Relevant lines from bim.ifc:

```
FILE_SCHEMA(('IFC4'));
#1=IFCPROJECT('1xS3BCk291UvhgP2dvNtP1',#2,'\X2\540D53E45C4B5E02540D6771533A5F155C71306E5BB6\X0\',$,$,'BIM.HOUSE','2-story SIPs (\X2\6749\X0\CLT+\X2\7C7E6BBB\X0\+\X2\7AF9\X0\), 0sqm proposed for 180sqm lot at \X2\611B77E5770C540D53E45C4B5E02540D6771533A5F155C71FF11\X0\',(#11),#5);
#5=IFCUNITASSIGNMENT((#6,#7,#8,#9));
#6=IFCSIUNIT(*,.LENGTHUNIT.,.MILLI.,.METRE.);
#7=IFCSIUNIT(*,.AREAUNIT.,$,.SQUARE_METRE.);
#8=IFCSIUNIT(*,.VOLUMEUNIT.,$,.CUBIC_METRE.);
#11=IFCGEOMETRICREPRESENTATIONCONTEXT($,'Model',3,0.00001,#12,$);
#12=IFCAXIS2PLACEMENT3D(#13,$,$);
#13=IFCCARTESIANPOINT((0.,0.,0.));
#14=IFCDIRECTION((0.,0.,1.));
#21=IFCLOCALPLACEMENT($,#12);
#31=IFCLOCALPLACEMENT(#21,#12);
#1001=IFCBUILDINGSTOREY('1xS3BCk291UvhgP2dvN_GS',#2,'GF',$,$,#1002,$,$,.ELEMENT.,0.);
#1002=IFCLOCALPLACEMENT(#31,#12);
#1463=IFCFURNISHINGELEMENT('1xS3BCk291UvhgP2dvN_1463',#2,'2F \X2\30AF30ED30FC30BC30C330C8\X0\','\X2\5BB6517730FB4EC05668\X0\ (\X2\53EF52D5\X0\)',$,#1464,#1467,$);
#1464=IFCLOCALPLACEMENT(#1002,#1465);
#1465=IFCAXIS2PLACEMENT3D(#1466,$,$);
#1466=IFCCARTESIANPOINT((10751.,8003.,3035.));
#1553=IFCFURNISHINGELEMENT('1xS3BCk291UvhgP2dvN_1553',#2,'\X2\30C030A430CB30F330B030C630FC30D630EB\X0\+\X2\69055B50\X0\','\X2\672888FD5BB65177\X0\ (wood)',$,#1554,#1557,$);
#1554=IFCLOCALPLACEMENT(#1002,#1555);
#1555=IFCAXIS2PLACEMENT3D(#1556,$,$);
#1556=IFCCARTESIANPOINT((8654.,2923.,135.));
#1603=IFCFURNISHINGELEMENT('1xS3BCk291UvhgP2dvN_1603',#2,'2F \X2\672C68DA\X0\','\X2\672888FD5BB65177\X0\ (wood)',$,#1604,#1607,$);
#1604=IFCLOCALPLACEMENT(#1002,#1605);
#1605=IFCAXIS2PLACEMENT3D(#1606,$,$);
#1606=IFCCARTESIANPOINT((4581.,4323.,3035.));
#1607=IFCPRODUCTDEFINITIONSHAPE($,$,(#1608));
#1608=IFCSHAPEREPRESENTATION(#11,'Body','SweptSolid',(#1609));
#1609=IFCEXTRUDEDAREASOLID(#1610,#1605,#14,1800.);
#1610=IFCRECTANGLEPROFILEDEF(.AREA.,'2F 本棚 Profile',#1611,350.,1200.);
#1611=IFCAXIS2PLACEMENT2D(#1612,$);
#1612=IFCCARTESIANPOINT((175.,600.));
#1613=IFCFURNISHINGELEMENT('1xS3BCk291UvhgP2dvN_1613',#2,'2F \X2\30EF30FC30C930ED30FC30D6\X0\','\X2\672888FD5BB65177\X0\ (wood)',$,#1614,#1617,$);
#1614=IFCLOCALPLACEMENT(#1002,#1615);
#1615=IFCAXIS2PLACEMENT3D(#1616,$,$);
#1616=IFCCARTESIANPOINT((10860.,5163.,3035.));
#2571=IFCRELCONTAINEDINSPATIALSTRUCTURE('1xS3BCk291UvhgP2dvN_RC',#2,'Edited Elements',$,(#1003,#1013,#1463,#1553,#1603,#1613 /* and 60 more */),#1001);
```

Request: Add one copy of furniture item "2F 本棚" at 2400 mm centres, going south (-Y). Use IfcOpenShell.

```python
import numpy as np
import ifcopenshell
import ifcopenshell.api.geometry
import ifcopenshell.api.root
import ifcopenshell.util.element
import ifcopenshell.util.placement

model = ifcopenshell.open("bim.ifc")


def reuse_history(source, copy):
    """copy_class also copies each property set's owner history, people and application; keep the originals."""
    for rel in copy.IsDefinedBy:
        if rel.is_a("IfcRelDefinesByProperties") and (history := rel.RelatingPropertyDefinition.OwnerHistory):
            rel.RelatingPropertyDefinition.OwnerHistory = source.OwnerHistory
            ifcopenshell.util.element.remove_deep2(model, history)


source = model.by_id(1603)
base = ifcopenshell.util.placement.get_local_placement(source.ObjectPlacement)
step = np.array([0.0, -1.0, 0.0]) * 2400.0

for i in range(1, 2):
    copy = ifcopenshell.api.root.copy_class(model, product=source)
    copy.Representation = ifcopenshell.util.element.copy_deep(
        model, source.Representation, exclude=["IfcGeometricRepresentationContext", "IfcRepresentationMap"]
    )
    reuse_history(source, copy)
    matrix = base.copy()
    matrix[:3, 3] += i * step
    print("added at", matrix[:3, 3].round(3) + 0.0)
    ifcopenshell.api.geometry.edit_object_placement(model, product=copy, matrix=matrix, is_si=False)

model.write("bim-out.ifc")
```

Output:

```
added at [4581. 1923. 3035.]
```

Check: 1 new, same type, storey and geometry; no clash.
